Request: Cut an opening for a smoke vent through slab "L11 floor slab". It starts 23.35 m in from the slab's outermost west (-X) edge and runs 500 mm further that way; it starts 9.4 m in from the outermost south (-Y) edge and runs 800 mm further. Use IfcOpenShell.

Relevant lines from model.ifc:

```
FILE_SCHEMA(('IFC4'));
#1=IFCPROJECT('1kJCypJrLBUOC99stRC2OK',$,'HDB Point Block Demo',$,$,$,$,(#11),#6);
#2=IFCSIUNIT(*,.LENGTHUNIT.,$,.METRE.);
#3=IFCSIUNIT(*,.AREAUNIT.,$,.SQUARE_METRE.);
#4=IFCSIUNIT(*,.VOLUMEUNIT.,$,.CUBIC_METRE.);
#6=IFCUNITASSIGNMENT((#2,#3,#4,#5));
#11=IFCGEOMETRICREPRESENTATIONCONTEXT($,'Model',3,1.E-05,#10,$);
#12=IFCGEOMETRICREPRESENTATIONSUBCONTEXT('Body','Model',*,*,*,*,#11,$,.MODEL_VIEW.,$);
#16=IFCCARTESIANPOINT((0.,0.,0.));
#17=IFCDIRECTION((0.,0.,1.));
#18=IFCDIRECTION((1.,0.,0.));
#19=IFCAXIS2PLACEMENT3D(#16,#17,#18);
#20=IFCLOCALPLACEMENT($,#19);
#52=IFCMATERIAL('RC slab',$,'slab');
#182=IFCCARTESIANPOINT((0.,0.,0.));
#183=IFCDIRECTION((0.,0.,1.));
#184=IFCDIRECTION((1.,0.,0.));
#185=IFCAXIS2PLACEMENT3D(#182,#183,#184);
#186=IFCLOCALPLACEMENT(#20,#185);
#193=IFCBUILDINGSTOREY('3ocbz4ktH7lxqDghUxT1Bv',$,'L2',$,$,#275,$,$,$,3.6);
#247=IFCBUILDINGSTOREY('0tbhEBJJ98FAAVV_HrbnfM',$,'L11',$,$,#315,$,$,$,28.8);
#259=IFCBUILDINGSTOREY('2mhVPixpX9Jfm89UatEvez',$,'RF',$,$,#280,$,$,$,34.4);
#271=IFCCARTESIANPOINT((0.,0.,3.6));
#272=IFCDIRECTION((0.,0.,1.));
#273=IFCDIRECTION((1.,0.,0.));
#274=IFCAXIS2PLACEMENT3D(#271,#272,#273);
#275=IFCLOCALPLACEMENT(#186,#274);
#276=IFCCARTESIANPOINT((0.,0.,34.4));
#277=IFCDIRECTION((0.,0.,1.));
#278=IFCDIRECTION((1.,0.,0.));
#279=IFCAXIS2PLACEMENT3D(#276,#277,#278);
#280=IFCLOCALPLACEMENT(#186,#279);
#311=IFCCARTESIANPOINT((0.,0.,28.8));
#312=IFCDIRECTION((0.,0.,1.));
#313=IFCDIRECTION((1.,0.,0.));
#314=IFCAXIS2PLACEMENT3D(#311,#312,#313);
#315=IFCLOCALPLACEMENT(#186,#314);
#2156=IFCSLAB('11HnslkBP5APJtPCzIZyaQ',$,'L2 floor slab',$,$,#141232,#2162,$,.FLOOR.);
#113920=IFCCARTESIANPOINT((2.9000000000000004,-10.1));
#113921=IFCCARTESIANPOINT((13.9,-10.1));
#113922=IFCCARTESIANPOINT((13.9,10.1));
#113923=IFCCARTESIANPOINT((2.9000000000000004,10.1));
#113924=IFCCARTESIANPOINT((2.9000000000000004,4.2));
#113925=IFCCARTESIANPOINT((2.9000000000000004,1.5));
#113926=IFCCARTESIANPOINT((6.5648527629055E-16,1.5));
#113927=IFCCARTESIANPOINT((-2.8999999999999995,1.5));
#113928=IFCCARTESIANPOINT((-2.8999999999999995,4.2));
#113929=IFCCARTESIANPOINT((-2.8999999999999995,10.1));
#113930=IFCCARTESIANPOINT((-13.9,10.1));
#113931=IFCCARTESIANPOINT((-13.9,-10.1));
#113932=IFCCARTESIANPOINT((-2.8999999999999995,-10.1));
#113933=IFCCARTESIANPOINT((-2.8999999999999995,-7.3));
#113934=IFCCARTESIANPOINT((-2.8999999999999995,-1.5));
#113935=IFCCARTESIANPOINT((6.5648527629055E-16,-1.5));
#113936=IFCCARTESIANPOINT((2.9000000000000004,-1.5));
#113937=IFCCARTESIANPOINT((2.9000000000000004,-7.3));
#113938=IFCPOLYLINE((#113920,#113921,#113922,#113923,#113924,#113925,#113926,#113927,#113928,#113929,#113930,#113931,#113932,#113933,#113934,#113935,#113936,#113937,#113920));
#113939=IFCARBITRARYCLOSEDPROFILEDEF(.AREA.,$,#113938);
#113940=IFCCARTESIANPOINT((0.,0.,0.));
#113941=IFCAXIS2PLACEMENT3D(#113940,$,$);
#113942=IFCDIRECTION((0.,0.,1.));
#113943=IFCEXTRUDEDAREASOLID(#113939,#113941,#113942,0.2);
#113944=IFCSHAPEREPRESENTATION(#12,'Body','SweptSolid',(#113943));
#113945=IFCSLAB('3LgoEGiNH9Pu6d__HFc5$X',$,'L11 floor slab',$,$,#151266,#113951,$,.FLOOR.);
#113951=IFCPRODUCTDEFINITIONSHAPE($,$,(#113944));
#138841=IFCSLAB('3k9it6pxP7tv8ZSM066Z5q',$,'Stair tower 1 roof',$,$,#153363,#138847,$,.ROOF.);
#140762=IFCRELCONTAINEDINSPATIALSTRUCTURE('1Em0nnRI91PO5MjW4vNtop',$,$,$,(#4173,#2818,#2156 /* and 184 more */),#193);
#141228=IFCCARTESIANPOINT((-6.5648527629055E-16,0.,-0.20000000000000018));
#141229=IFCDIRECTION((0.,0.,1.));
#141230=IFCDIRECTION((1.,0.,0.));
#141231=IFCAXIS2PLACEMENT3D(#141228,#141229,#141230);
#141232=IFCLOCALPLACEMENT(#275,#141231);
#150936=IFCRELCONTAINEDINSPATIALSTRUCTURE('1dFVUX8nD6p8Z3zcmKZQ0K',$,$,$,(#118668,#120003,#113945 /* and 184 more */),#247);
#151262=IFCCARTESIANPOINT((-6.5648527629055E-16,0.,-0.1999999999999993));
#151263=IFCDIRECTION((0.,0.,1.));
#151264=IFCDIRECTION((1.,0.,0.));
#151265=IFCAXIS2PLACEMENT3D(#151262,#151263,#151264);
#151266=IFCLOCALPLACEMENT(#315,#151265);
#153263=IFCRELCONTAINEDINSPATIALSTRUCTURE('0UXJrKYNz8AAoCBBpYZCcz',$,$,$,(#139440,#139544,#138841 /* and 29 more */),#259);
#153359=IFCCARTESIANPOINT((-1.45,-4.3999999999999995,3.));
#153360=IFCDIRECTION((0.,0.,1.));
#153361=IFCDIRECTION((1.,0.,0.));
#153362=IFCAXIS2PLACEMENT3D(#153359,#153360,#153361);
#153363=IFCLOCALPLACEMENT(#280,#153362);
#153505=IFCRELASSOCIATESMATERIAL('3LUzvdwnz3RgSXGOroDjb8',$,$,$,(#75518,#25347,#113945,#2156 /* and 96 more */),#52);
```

```python
import numpy as np
import ifcopenshell
import ifcopenshell.api.feature
import ifcopenshell.api.geometry
import ifcopenshell.api.root
import ifcopenshell.geom
import ifcopenshell.util.placement
import ifcopenshell.util.representation
import ifcopenshell.util.shape
import ifcopenshell.util.unit

model = ifcopenshell.open("model.ifc")
unit_scale = ifcopenshell.util.unit.calculate_unit_scale(model)
settings = ifcopenshell.geom.settings()


def volume(element):
    """Net volume in cubic metres, openings subtracted."""
    shape = ifcopenshell.geom.create_shape(settings, element)
    return ifcopenshell.util.shape.get_volume(shape.geometry)


slab = model.by_guid("3LgoEGiNH9Pu6d__HFc5$X")
before = volume(slab)

# Extent in the slab's own axes, in metres. The edges named are its -X and -Y sides.
slab_shape = ifcopenshell.geom.create_shape(settings, slab)
vertices = ifcopenshell.util.shape.get_vertices(slab_shape.geometry)
x_min, y_min, bottom = vertices.min(axis=0)
top = vertices[:, 2].max()

opening = ifcopenshell.api.root.create_entity(model, ifc_class="IfcOpeningElement", name="Smoke vent opening", predefined_type="OPENING")
context = ifcopenshell.util.representation.get_context(model, "Model", "Body", "MODEL_VIEW")
width, depth = 0.5, 0.8
outline = [(0.0, 0.0), (width, 0.0), (width, depth), (0.0, depth), (0.0, 0.0)]
# Overshoot both faces by 50 mm so the cut is clean.
shape = ifcopenshell.api.geometry.add_slab_representation(
    model, context=context, depth=top - bottom + 0.1, polyline=outline
)
ifcopenshell.api.geometry.assign_representation(model, product=opening, representation=shape)

matrix = ifcopenshell.util.placement.get_local_placement(slab.ObjectPlacement)
matrix[:, 3] = matrix @ np.append(np.array([x_min + 23.35, y_min + 9.4, bottom - 0.05]) / unit_scale, 1.0)
ifcopenshell.api.geometry.edit_object_placement(model, product=opening, matrix=matrix, is_si=False)
ifcopenshell.api.feature.add_feature(model, feature=opening, element=slab)

after = volume(slab)

print(f"slab volume {before:.3f} -> {after:.3f} m3")

model.write("model-out.ifc")
```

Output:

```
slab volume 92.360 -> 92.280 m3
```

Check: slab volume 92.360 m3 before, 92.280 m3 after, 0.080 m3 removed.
